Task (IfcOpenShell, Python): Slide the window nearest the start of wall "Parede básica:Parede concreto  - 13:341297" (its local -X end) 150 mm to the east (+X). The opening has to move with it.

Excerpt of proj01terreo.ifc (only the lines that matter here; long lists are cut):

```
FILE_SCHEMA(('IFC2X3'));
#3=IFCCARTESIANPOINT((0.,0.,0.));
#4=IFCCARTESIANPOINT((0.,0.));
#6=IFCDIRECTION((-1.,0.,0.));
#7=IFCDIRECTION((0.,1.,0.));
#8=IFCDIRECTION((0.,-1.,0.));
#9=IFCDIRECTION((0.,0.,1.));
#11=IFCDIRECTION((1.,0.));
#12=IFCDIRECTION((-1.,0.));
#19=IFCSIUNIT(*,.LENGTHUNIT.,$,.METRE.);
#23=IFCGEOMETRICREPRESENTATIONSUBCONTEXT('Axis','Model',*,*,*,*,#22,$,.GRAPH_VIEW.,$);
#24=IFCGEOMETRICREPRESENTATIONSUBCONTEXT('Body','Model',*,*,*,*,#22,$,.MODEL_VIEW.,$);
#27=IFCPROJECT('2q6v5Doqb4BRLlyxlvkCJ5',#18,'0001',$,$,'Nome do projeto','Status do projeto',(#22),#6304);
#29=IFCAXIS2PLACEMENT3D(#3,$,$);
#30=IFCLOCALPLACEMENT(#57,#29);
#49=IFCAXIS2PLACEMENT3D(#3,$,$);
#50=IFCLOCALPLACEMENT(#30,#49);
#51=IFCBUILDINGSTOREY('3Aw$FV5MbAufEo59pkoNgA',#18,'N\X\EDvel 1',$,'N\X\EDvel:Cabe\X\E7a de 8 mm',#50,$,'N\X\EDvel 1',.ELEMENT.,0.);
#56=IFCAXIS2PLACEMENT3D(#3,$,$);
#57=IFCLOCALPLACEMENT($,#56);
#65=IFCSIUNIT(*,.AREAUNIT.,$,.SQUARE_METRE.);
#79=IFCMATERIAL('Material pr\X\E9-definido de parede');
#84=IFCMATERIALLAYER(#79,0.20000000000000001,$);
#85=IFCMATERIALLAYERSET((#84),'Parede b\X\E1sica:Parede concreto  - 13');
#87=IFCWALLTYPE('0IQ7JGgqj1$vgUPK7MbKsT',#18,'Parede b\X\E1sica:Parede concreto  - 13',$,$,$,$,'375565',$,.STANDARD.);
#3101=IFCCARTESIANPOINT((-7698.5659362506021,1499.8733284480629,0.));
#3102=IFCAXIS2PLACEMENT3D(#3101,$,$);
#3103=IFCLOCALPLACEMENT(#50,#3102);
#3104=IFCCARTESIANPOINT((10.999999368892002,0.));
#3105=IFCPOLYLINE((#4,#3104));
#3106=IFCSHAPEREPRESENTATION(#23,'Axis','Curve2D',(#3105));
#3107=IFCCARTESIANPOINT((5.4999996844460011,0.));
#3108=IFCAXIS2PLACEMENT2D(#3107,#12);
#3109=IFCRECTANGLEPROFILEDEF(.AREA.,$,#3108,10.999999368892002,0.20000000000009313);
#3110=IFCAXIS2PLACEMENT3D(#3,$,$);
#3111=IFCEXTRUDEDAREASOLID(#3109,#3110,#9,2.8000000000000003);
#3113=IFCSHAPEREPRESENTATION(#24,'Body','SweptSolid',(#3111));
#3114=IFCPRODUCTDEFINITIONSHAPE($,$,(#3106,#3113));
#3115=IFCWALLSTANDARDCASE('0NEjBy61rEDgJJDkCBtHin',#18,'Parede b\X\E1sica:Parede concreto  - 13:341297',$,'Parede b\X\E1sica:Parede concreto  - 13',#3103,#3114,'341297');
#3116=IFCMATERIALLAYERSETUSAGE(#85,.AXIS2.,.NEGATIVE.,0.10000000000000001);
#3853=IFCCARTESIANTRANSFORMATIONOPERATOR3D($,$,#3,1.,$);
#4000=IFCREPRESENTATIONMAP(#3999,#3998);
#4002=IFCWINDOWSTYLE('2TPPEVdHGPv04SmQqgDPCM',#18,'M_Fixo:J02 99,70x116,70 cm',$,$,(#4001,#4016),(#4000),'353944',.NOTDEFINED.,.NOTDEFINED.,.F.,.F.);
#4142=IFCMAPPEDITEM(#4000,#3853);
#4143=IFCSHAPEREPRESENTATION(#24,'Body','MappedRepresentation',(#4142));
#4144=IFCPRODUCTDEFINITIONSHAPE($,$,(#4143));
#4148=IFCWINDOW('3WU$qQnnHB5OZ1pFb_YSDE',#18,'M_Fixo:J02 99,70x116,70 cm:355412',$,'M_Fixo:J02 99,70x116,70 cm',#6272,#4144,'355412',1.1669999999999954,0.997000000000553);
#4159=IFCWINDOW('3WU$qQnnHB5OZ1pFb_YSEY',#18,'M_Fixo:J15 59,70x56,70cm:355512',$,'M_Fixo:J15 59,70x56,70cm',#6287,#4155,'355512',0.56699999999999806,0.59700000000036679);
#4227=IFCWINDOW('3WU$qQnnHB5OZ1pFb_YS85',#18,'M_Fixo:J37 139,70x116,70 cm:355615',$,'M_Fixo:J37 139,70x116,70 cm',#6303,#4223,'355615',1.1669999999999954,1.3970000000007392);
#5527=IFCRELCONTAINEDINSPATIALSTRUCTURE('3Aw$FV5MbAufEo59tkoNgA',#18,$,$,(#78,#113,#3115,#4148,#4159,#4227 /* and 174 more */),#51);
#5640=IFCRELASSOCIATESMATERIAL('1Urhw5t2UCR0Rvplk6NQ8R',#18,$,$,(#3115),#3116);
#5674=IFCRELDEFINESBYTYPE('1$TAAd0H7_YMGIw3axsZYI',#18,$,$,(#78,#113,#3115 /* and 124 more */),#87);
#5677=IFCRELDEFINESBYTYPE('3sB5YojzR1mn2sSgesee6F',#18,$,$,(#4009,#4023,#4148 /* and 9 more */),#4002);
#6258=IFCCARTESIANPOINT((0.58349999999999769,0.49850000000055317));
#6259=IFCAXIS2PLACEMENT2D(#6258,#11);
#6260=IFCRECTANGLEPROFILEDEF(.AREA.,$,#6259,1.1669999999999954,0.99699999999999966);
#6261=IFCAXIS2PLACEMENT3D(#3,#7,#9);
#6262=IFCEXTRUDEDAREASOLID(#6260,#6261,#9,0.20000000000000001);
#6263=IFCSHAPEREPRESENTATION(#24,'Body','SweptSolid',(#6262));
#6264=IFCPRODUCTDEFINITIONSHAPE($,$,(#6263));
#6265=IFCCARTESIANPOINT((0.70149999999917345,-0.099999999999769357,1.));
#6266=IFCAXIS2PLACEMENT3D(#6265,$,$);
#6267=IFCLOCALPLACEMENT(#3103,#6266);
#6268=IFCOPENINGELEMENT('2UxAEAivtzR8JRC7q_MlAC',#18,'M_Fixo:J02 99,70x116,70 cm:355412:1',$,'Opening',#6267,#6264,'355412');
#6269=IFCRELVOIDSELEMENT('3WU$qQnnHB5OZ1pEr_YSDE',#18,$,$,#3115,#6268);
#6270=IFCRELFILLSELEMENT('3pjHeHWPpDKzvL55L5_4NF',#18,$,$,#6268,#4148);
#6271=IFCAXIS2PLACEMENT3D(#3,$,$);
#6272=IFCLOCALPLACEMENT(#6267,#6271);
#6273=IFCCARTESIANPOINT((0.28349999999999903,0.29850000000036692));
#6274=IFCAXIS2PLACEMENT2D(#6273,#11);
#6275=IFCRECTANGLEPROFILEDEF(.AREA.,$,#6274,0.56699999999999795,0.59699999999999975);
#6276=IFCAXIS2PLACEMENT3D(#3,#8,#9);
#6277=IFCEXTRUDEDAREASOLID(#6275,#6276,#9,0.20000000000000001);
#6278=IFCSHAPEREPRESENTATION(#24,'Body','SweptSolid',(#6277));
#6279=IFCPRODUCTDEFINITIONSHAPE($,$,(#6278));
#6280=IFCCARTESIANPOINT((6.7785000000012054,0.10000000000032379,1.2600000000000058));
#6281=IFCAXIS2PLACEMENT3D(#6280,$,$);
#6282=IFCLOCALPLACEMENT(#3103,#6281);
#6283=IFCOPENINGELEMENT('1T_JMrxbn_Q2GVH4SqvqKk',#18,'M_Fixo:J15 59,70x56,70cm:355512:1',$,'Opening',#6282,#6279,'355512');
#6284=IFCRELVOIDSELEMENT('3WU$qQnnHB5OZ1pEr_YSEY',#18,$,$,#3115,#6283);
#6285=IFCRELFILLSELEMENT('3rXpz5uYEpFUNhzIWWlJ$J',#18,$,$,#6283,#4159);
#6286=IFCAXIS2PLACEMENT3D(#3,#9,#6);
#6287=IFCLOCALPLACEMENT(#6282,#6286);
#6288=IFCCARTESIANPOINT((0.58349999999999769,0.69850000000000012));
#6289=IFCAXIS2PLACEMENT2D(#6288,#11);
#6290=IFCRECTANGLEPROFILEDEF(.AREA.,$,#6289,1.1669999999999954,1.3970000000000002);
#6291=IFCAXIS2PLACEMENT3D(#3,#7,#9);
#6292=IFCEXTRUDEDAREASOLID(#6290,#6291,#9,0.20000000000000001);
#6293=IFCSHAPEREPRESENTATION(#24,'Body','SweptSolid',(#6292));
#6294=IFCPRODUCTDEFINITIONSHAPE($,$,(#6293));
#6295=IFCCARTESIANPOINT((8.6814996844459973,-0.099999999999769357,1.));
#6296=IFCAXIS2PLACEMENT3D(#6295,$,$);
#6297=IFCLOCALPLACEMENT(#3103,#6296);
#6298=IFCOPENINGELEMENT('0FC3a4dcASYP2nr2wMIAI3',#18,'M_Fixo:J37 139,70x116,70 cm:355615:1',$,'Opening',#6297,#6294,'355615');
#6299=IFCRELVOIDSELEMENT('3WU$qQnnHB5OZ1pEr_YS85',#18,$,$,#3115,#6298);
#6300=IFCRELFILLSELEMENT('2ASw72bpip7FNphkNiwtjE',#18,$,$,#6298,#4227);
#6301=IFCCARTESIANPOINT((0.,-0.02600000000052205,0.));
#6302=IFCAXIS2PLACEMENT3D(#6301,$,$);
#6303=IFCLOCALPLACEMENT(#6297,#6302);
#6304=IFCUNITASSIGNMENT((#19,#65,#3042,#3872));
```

```python
import ifcopenshell
import ifcopenshell.api.geometry
import ifcopenshell.util.placement
import ifcopenshell.util.unit

model = ifcopenshell.open("proj01terreo.ifc")
unit_scale = ifcopenshell.util.unit.calculate_unit_scale(model)

window = model.by_guid("3WU$qQnnHB5OZ1pFb_YSDE")
opening = window.FillsVoids[0].RelatingOpeningElement
wall = opening.VoidsElements[0].RelatingBuildingElement

wall_matrix = ifcopenshell.util.placement.get_local_placement(wall.ObjectPlacement)
shift = wall_matrix[:3, 0] * 0.15 / unit_scale
before = ifcopenshell.util.placement.get_local_placement(window.ObjectPlacement)[:3, 3].copy()

# The window is placed relative to its opening, so it follows when the opening moves.
matrix = ifcopenshell.util.placement.get_local_placement(opening.ObjectPlacement)
matrix[:3, 3] += shift
ifcopenshell.api.geometry.edit_object_placement(
    model, product=opening, matrix=matrix, is_si=False, should_transform_children=True
)

after = ifcopenshell.util.placement.get_local_placement(window.ObjectPlacement)[:3, 3]
print("window moved by", (after - before).round(3) + 0.0)

model.write("proj01terreo_rev.ifc")
```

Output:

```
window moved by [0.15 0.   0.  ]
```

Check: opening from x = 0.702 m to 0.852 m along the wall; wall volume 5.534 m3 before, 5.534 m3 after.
